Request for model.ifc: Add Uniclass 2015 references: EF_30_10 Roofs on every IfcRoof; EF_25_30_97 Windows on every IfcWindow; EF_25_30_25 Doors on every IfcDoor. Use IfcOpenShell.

First a look at what the model holds.

```python
import ifcopenshell

model = ifcopenshell.open("model.ifc")
print(model.schema)
print("classifications:", [c.Name for c in model.by_type("IfcClassification")])
for ifc_class in ("IfcDoor", "IfcRoof", "IfcStair", "IfcWall", "IfcWindow"):
    print(ifc_class, len(model.by_type(ifc_class)))
```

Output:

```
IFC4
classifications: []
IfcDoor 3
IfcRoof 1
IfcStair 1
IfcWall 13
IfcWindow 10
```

```python
import ifcopenshell
import ifcopenshell.api.classification

model = ifcopenshell.open("model.ifc")

system = ifcopenshell.api.classification.add_classification(model, classification="Uniclass 2015")

codes = {
    "IfcRoof": ("EF_30_10", "Roofs"),
    "IfcWindow": ("EF_25_30_97", "Windows"),
    "IfcDoor": ("EF_25_30_25", "Doors"),
}
for ifc_class, (code, name) in codes.items():
    products = model.by_type(ifc_class)
    ifcopenshell.api.classification.add_reference(
        model, products=products, classification=system, identification=code, name=name
    )
    print(code, len(products))

model.write("model_edited.ifc")
```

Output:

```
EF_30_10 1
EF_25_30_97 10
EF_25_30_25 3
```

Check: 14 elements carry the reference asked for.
